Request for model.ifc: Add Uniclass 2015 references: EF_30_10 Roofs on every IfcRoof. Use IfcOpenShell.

First a look at what the model holds.

```python
import ifcopenshell

model = ifcopenshell.open("model.ifc")
print(model.schema)
print("classifications:", [c.Name for c in model.by_type("IfcClassification")])
for ifc_class in ("IfcDoor", "IfcRoof", "IfcStair", "IfcWall", "IfcWindow"):
    print(ifc_class, len(model.by_type(ifc_class)))
```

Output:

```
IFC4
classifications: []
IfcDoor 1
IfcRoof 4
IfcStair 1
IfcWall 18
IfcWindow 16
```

```python
import ifcopenshell
import ifcopenshell.api.classification

model = ifcopenshell.open("model.ifc")

system = ifcopenshell.api.classification.add_classification(model, classification="Uniclass 2015")

codes = {
    "IfcRoof": ("EF_30_10", "Roofs"),
}
for ifc_class, (code, name) in codes.items():
    products = model.by_type(ifc_class)
    ifcopenshell.api.classification.add_reference(
        model, products=products, classification=system, identification=code, name=name
    )
    print(code, len(products))

model.write("model-out.ifc")
```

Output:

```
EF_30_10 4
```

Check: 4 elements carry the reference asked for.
